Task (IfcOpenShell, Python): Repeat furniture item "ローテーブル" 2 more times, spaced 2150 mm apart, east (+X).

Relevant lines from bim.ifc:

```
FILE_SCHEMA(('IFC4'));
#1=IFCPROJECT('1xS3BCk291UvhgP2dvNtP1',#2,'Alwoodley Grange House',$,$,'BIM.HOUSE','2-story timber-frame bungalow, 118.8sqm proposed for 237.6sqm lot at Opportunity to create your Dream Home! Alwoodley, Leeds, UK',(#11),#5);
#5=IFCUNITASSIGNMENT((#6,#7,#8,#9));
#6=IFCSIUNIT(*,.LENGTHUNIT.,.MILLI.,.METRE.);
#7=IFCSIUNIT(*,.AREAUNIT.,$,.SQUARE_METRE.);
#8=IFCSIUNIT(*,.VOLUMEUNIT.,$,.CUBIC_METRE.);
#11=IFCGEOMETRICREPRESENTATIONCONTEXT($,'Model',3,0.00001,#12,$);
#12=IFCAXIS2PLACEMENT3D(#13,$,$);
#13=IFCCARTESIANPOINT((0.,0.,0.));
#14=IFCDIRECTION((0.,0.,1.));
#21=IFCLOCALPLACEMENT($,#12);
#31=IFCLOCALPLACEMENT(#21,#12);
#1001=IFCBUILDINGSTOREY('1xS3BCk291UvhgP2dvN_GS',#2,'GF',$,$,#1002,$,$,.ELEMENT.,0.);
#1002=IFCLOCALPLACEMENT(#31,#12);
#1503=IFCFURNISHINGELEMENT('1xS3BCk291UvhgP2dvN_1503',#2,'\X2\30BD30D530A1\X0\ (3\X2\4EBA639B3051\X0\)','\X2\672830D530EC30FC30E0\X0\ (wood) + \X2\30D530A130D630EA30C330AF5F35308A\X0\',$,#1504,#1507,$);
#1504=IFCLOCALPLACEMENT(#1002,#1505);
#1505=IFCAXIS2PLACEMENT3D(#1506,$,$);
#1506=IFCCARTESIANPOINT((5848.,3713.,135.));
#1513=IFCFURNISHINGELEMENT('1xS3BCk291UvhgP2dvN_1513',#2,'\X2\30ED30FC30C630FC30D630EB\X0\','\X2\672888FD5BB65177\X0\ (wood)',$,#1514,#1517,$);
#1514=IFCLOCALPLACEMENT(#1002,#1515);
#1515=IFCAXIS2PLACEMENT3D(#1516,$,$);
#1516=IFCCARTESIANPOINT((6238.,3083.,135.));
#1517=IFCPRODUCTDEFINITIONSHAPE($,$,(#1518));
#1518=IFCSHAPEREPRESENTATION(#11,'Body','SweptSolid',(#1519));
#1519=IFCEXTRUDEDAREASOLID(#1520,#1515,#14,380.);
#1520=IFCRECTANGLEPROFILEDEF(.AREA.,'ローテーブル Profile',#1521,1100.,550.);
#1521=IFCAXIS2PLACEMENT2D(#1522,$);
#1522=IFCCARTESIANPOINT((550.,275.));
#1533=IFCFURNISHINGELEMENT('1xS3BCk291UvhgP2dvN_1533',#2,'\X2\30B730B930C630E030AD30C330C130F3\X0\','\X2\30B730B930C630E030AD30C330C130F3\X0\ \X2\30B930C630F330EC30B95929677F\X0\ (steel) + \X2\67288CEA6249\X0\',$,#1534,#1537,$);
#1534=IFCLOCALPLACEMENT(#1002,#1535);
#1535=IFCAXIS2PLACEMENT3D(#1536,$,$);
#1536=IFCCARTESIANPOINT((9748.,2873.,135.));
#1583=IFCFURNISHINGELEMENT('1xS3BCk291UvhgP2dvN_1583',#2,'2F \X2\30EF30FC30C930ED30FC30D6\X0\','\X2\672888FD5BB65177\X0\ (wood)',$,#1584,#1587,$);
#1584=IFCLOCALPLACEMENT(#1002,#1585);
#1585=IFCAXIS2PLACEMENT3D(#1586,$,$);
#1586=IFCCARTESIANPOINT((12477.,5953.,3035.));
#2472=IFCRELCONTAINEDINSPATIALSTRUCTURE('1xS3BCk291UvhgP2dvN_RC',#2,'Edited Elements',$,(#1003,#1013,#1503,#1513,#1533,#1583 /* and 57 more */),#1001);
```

```python
import numpy as np
import ifcopenshell
import ifcopenshell.api.geometry
import ifcopenshell.api.root
import ifcopenshell.util.element
import ifcopenshell.util.placement

model = ifcopenshell.open("bim.ifc")


def reuse_history(source, copy):
    """copy_class also copies each property set's owner history, people and application; keep the originals."""
    for rel in copy.IsDefinedBy:
        if rel.is_a("IfcRelDefinesByProperties") and (history := rel.RelatingPropertyDefinition.OwnerHistory):
            rel.RelatingPropertyDefinition.OwnerHistory = source.OwnerHistory
            ifcopenshell.util.element.remove_deep2(model, history)


source = model.by_guid("1xS3BCk291UvhgP2dvN_1513")
base = ifcopenshell.util.placement.get_local_placement(source.ObjectPlacement)
step = np.array([1.0, 0.0, 0.0]) * 2150.0

for i in range(1, 3):
    copy = ifcopenshell.api.root.copy_class(model, product=source)
    copy.Representation = ifcopenshell.util.element.copy_deep(
        model, source.Representation, exclude=["IfcGeometricRepresentationContext", "IfcRepresentationMap"]
    )
    reuse_history(source, copy)
    matrix = base.copy()
    matrix[:3, 3] += i * step
    print("added at", matrix[:3, 3].round(3) + 0.0)
    ifcopenshell.api.geometry.edit_object_placement(model, product=copy, matrix=matrix, is_si=False)

model.write("bim_rev.ifc")
```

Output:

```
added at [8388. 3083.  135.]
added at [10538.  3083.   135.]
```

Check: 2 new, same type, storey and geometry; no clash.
